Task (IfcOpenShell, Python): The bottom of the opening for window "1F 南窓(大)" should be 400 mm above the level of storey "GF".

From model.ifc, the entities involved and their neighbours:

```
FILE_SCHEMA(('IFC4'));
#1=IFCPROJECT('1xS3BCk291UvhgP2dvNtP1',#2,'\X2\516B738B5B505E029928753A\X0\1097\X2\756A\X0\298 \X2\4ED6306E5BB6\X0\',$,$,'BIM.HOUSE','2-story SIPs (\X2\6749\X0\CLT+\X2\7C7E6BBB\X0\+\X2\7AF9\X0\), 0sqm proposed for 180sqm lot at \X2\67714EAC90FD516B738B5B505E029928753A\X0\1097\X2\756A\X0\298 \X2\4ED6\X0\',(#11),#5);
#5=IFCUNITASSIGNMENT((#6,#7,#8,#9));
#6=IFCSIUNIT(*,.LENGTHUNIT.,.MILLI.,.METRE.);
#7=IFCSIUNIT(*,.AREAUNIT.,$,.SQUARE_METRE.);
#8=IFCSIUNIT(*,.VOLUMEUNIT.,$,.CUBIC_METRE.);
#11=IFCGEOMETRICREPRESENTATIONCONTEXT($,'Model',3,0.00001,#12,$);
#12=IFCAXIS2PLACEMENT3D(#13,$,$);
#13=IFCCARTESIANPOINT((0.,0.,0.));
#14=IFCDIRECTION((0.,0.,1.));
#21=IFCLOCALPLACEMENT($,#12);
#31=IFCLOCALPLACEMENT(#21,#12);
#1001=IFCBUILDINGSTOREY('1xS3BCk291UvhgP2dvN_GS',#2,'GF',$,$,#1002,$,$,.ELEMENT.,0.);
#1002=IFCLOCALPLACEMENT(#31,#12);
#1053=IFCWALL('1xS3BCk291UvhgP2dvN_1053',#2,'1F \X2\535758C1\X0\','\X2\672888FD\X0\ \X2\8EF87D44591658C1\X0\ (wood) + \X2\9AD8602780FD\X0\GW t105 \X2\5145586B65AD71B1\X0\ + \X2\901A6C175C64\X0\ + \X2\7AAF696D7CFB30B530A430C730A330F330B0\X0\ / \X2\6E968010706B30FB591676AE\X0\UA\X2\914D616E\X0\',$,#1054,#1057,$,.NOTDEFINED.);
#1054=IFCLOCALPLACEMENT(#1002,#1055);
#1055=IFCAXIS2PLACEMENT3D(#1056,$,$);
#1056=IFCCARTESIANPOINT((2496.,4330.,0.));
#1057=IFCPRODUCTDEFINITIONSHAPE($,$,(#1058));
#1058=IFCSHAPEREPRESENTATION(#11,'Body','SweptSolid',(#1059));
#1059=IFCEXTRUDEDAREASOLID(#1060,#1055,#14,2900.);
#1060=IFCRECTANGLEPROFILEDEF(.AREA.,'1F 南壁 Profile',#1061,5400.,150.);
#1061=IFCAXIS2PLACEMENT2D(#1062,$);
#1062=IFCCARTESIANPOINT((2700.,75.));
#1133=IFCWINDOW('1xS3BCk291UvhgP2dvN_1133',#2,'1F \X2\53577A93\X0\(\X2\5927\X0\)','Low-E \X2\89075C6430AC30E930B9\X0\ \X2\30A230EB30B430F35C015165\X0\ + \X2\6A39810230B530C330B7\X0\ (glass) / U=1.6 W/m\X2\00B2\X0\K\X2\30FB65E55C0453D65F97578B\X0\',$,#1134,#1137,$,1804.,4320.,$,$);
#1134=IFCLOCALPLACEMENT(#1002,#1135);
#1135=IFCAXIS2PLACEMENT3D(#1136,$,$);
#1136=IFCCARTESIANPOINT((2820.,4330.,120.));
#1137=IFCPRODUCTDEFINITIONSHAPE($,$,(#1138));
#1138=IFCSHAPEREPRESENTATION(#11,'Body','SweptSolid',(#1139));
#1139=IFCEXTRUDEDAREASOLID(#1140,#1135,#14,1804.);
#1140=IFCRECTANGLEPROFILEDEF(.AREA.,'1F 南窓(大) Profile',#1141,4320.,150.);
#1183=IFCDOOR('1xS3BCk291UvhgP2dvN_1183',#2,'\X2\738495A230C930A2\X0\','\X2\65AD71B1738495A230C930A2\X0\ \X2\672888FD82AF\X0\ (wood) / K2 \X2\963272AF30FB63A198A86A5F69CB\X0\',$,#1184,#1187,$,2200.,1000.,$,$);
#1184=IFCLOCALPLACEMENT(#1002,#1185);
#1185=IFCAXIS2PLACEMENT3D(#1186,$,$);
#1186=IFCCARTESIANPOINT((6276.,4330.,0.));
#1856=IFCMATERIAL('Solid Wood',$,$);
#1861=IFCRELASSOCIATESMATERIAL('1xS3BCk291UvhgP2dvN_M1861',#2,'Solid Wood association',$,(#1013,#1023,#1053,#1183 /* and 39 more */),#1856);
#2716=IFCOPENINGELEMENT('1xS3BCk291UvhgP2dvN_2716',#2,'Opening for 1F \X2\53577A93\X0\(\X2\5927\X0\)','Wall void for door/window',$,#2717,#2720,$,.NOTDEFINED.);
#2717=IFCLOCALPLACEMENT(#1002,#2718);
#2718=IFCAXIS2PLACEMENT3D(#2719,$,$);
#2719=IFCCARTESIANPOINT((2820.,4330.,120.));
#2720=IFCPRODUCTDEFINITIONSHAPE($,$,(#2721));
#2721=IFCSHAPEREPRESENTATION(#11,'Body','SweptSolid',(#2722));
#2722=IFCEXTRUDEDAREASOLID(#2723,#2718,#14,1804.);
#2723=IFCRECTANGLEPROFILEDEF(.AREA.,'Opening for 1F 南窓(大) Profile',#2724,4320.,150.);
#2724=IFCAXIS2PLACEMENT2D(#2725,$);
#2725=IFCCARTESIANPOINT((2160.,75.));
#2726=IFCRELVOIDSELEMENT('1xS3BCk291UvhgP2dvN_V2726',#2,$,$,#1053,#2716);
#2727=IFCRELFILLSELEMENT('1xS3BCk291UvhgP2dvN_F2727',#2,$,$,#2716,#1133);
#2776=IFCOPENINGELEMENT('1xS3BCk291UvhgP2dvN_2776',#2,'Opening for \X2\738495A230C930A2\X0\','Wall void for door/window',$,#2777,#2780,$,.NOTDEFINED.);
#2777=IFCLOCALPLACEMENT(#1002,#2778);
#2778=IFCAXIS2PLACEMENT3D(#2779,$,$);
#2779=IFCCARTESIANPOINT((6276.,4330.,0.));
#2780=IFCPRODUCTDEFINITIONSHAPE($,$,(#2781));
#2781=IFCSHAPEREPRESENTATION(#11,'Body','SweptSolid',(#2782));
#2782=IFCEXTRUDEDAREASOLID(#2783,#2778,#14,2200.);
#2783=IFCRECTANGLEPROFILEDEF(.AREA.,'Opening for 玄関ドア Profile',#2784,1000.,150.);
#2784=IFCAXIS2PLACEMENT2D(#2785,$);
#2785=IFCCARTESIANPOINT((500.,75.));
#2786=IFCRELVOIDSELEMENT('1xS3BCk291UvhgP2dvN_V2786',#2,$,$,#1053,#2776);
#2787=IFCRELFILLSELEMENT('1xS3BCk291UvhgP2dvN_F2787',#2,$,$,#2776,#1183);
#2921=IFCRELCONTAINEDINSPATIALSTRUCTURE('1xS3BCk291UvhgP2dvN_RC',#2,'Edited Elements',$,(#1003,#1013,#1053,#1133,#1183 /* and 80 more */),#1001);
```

```python
import numpy as np
import ifcopenshell
import ifcopenshell.api.geometry
import ifcopenshell.geom
import ifcopenshell.util.element
import ifcopenshell.util.placement
import ifcopenshell.util.shape
import ifcopenshell.util.unit

model = ifcopenshell.open("model.ifc")
unit_scale = ifcopenshell.util.unit.calculate_unit_scale(model)

window = model.by_guid("1xS3BCk291UvhgP2dvN_1133")
opening = window.FillsVoids[0].RelatingOpeningElement
storey = ifcopenshell.util.element.get_container(window, ifc_class="IfcBuildingStorey")
level = ifcopenshell.util.placement.get_local_placement(storey.ObjectPlacement)[2, 3]

# The opening's origin need not be at the sill, so measure its lowest point.
shape = ifcopenshell.geom.create_shape(ifcopenshell.geom.settings(), opening)
bottom = ifcopenshell.util.shape.get_shape_bottom_elevation(shape, shape.geometry) / unit_scale
dz = level + 0.4 / unit_scale - bottom

shift = np.array([0.0, 0.0, dz])
# The window is not placed relative to its opening, so move both.
for product in (opening, window):
    matrix = ifcopenshell.util.placement.get_local_placement(product.ObjectPlacement)
    matrix[:3, 3] += shift
    ifcopenshell.api.geometry.edit_object_placement(model, product=product, matrix=matrix, is_si=False)

print(f"moved by {dz * unit_scale:+.3f} m")

model.write("model_v2.ifc")
```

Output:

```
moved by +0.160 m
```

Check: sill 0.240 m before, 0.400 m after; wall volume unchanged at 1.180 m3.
